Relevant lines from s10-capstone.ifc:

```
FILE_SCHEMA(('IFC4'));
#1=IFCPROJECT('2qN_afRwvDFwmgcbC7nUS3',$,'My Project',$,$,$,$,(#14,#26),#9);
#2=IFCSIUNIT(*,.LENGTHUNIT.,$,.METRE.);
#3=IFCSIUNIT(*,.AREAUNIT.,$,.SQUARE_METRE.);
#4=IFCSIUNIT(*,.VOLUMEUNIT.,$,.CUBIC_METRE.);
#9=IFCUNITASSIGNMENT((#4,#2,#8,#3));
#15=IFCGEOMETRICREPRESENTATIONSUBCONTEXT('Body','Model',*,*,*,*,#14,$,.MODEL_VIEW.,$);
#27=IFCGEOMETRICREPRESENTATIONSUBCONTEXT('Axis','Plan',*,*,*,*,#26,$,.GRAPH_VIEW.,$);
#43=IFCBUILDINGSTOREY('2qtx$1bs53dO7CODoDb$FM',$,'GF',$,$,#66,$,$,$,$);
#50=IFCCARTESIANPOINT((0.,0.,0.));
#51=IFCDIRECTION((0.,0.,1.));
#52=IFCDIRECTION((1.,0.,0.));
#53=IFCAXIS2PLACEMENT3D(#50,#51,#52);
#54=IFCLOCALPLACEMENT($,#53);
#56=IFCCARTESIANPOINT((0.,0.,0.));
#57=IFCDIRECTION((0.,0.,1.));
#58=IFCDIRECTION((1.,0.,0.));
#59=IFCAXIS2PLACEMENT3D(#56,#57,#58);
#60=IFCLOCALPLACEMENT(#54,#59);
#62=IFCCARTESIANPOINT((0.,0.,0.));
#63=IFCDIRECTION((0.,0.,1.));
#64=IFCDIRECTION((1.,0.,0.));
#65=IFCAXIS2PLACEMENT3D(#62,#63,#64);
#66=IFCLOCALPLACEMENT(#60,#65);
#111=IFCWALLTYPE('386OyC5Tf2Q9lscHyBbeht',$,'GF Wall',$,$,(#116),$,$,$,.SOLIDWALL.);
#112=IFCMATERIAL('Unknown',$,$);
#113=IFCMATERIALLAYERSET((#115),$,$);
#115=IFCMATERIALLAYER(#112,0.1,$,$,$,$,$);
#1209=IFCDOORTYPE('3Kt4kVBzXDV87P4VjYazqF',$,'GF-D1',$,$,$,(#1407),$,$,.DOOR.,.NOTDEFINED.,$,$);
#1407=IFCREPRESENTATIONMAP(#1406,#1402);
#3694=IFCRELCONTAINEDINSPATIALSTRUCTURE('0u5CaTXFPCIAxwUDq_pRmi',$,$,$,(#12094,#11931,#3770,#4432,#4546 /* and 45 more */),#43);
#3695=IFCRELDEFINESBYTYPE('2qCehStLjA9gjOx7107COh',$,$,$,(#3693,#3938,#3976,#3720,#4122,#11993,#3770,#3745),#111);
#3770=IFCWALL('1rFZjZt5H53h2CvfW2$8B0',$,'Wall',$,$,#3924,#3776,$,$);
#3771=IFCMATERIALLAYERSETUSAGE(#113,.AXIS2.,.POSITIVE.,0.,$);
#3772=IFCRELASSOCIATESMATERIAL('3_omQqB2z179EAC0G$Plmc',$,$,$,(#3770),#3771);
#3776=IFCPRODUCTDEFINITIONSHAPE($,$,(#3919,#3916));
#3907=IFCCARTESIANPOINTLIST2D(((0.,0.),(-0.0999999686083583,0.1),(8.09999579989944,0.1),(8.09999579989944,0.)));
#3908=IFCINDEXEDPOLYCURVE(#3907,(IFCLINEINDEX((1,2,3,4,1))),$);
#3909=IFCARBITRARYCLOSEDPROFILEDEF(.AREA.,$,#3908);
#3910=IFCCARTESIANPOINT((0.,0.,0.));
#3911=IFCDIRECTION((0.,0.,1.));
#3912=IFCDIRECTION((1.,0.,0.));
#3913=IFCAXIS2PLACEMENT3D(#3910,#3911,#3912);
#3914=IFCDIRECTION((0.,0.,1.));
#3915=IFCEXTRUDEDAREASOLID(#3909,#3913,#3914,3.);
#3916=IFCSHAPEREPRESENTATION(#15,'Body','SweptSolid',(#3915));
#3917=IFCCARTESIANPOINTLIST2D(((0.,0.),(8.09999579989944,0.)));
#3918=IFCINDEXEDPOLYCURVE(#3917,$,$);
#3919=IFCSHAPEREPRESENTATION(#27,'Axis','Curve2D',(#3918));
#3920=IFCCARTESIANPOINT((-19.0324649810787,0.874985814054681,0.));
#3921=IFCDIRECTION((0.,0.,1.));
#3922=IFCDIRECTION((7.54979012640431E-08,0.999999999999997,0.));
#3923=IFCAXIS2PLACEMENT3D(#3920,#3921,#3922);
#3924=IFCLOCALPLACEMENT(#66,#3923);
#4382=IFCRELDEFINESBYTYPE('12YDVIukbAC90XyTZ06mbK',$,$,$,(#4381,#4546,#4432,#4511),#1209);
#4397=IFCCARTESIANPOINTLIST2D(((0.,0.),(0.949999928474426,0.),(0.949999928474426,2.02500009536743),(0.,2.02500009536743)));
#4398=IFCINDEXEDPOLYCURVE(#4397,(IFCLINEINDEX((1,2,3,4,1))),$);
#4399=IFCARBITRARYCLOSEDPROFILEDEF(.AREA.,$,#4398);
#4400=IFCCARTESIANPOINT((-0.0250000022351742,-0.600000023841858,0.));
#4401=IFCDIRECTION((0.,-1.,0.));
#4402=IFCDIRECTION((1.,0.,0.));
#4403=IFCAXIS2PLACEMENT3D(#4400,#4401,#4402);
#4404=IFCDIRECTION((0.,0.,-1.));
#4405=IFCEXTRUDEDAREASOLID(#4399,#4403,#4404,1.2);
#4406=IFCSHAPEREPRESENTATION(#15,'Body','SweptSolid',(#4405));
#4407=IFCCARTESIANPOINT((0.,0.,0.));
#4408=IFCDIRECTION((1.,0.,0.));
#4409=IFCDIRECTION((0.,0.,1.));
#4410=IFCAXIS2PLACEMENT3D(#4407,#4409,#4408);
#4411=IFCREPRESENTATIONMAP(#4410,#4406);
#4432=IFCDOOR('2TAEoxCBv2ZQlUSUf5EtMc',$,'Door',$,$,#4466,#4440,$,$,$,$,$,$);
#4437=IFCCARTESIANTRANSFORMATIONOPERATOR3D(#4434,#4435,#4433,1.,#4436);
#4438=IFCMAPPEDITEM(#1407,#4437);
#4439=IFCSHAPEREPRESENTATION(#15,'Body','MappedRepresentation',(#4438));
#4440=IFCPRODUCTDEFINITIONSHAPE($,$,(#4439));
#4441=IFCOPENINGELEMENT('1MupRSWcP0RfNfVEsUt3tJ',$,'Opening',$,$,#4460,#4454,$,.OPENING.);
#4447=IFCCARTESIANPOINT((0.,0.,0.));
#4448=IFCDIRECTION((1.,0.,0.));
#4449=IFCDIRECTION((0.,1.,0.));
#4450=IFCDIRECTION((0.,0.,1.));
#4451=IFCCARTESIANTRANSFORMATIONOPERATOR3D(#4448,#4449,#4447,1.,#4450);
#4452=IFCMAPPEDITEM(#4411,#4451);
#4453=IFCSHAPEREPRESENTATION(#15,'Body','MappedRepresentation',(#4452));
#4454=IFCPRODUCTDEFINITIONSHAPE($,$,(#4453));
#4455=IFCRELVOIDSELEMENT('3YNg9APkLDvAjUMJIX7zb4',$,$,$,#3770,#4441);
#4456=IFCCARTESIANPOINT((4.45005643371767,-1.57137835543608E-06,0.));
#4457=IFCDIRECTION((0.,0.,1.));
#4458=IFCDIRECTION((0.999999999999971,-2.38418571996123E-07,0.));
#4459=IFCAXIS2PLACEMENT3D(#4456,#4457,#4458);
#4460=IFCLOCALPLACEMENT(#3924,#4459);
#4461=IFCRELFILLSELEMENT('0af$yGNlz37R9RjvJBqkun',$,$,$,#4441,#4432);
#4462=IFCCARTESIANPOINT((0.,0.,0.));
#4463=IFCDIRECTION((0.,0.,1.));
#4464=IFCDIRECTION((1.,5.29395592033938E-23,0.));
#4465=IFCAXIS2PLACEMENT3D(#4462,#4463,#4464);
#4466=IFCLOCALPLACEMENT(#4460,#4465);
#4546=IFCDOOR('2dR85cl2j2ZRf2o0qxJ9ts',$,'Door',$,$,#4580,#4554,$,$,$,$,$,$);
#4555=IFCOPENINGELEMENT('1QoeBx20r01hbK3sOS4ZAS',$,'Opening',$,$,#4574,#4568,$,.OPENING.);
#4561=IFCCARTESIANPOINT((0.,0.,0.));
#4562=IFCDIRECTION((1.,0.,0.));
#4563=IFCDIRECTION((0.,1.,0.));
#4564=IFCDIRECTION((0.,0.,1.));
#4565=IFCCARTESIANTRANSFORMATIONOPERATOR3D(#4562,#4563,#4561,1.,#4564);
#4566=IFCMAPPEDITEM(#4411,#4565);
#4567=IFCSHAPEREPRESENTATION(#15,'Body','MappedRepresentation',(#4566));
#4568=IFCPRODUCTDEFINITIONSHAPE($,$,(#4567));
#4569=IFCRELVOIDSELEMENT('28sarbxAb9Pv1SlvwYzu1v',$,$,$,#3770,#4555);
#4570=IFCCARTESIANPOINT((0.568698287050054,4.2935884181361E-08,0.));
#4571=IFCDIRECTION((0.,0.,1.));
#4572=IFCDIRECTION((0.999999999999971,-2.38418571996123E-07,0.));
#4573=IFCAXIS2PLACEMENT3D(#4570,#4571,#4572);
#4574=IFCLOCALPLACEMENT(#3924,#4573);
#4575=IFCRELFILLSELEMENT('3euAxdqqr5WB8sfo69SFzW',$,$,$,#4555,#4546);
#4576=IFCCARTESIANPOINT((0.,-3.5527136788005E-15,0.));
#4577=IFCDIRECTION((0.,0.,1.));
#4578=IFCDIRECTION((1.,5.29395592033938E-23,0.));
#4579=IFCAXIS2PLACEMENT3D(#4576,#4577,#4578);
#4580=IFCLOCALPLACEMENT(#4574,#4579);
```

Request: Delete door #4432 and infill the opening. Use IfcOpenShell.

```python
import ifcopenshell
import ifcopenshell.api.feature
import ifcopenshell.api.root
import ifcopenshell.geom
import ifcopenshell.util.shape

model = ifcopenshell.open("s10-capstone.ifc")
settings = ifcopenshell.geom.settings()


def volume(element):
    """Net volume in cubic metres, openings subtracted."""
    shape = ifcopenshell.geom.create_shape(settings, element)
    return ifcopenshell.util.shape.get_volume(shape.geometry)


door = model.by_id(4432)
opening = door.FillsVoids[0].RelatingOpeningElement
wall = opening.VoidsElements[0].RelatingBuildingElement
before = volume(wall)

ifcopenshell.api.root.remove_product(model, product=door)
ifcopenshell.api.feature.remove_feature(model, feature=opening)

after = volume(wall)

print(f"wall volume {before:.3f} -> {after:.3f} m3")

model.write("s10-capstone_rev.ifc")
```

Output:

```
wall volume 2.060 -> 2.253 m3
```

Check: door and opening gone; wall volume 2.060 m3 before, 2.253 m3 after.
